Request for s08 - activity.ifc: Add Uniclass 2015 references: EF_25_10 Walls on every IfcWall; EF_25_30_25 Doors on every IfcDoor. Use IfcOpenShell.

First a look at what the model holds.

```python
import ifcopenshell

model = ifcopenshell.open("s08 - activity.ifc")
print(model.schema)
print("classifications:", [c.Name for c in model.by_type("IfcClassification")])
for ifc_class in ("IfcDoor", "IfcRoof", "IfcStair", "IfcWall", "IfcWindow"):
    print(ifc_class, len(model.by_type(ifc_class)))
```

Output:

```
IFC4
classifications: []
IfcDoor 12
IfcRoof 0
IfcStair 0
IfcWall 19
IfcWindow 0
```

```python
import ifcopenshell
import ifcopenshell.api.classification

model = ifcopenshell.open("s08 - activity.ifc")

system = ifcopenshell.api.classification.add_classification(model, classification="Uniclass 2015")

codes = {
    "IfcWall": ("EF_25_10", "Walls"),
    "IfcDoor": ("EF_25_30_25", "Doors"),
}
for ifc_class, (code, name) in codes.items():
    products = model.by_type(ifc_class)
    ifcopenshell.api.classification.add_reference(
        model, products=products, classification=system, identification=code, name=name
    )
    print(code, len(products))

model.write("s08 - activity_edited.ifc")
```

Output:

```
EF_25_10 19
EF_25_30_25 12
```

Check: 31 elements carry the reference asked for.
